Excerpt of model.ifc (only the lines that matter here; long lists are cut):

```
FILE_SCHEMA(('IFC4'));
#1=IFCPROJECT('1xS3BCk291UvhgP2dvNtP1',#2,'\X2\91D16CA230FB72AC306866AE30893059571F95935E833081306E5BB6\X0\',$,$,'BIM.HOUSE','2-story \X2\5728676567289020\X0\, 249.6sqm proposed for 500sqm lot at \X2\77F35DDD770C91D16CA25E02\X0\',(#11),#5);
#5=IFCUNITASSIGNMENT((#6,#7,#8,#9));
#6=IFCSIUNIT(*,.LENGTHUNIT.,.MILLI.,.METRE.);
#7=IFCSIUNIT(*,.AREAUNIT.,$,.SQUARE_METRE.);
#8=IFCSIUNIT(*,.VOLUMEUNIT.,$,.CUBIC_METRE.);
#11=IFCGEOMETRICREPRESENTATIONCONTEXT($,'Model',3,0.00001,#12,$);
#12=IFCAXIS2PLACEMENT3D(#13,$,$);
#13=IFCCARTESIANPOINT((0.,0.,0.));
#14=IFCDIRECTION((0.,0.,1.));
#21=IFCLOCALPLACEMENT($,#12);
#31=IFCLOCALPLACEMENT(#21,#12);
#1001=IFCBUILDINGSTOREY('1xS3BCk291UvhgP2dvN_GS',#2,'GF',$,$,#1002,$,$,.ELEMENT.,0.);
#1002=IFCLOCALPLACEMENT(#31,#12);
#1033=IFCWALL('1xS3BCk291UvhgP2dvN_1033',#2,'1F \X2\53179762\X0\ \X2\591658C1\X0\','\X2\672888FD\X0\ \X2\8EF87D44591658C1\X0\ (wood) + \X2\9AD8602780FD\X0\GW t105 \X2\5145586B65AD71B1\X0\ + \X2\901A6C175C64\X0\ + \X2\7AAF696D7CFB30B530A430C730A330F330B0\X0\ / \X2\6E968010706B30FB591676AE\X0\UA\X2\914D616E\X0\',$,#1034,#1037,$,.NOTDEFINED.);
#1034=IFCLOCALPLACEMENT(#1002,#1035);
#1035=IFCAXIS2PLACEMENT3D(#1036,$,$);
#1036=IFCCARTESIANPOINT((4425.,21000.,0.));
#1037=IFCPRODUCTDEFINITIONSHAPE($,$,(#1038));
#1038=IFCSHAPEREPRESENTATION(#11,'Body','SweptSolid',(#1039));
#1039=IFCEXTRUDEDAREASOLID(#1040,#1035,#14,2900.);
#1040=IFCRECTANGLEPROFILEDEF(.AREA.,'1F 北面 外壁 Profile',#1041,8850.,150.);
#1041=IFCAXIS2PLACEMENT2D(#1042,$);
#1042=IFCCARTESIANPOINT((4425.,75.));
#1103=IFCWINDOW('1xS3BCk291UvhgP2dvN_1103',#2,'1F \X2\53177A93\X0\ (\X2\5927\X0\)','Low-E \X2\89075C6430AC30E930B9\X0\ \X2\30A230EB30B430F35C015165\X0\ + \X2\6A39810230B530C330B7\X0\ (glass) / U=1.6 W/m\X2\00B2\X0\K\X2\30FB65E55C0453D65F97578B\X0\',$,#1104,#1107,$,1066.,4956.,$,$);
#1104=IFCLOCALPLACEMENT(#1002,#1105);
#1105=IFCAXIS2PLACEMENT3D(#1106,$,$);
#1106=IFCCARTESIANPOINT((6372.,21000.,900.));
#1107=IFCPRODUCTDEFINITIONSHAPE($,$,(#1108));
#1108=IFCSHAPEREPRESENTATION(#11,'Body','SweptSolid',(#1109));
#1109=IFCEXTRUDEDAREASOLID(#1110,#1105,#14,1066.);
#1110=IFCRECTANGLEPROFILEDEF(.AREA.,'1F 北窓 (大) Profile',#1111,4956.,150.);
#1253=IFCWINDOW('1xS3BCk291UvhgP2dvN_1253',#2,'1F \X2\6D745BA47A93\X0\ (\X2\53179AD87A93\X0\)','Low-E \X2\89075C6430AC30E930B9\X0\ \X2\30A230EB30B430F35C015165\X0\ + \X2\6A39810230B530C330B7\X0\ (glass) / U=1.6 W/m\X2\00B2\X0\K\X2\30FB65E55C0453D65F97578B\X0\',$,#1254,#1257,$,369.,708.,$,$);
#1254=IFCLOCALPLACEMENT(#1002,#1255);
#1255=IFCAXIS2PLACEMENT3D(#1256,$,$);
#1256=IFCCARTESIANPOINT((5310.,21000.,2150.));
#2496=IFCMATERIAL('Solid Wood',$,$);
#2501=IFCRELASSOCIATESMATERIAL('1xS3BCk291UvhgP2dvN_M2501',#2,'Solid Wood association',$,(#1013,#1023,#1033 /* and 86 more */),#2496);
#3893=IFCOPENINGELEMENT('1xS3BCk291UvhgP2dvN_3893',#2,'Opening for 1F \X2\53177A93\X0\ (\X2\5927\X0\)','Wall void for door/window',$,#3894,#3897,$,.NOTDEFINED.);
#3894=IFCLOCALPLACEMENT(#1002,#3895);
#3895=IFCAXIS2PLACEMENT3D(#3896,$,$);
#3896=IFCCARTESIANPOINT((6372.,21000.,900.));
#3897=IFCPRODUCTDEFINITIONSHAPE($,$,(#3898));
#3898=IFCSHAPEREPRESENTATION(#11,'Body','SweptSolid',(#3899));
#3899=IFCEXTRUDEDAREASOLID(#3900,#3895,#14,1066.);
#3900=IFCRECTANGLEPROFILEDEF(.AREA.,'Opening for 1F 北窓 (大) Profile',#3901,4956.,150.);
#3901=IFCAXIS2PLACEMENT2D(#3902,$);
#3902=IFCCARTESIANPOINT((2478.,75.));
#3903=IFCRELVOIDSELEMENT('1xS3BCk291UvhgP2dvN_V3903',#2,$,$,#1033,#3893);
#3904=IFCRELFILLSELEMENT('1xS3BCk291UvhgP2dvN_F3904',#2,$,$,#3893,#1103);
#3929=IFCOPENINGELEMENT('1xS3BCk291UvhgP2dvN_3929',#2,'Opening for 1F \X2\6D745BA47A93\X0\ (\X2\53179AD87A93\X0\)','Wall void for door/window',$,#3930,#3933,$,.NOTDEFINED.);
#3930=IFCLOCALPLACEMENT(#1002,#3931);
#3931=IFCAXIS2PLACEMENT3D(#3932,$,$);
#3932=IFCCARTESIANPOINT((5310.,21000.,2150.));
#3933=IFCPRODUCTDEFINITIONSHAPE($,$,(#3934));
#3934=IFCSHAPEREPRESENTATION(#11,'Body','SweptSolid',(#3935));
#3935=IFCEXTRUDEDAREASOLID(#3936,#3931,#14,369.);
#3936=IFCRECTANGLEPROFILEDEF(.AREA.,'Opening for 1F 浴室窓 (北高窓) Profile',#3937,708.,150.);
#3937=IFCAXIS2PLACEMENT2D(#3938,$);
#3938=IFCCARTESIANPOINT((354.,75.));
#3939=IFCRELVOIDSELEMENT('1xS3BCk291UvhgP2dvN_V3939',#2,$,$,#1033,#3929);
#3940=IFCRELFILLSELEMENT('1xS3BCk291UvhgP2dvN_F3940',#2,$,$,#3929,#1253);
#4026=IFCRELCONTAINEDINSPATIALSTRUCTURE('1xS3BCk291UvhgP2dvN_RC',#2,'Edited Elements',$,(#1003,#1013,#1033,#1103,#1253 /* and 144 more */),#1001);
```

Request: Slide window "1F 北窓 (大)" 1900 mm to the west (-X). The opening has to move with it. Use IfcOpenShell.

```python
import ifcopenshell
import ifcopenshell.api.geometry
import ifcopenshell.util.placement

model = ifcopenshell.open("model.ifc")

window = model.by_guid("1xS3BCk291UvhgP2dvN_1103")
opening = window.FillsVoids[0].RelatingOpeningElement
wall = opening.VoidsElements[0].RelatingBuildingElement

wall_matrix = ifcopenshell.util.placement.get_local_placement(wall.ObjectPlacement)
shift = wall_matrix[:3, 0] * -1900.0
before = ifcopenshell.util.placement.get_local_placement(window.ObjectPlacement)[:3, 3].copy()

# The window is not placed relative to its opening, so move both.
for product in (opening, window):
    matrix = ifcopenshell.util.placement.get_local_placement(product.ObjectPlacement)
    matrix[:3, 3] += shift
    ifcopenshell.api.geometry.edit_object_placement(model, product=product, matrix=matrix, is_si=False)

after = ifcopenshell.util.placement.get_local_placement(window.ObjectPlacement)[:3, 3]
print("window moved by", (after - before).round(3) + 0.0)

model.write("model-out.ifc")
```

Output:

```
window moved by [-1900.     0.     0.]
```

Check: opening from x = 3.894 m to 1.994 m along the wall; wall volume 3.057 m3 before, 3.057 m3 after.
